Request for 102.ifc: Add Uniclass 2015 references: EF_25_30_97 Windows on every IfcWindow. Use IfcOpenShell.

First a look at what the model holds.

```python
import ifcopenshell

model = ifcopenshell.open("102.ifc")
print(model.schema)
print("classifications:", [c.Name for c in model.by_type("IfcClassification")])
for ifc_class in ("IfcDoor", "IfcRoof", "IfcStair", "IfcWall", "IfcWindow"):
    print(ifc_class, len(model.by_type(ifc_class)))
```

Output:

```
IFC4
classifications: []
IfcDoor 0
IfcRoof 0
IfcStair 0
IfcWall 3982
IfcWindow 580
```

```python
import ifcopenshell
import ifcopenshell.api.classification

model = ifcopenshell.open("102.ifc")

system = ifcopenshell.api.classification.add_classification(model, classification="Uniclass 2015")

codes = {
    "IfcWindow": ("EF_25_30_97", "Windows"),
}
for ifc_class, (code, name) in codes.items():
    products = model.by_type(ifc_class)
    ifcopenshell.api.classification.add_reference(
        model, products=products, classification=system, identification=code, name=name
    )
    print(code, len(products))

model.write("102_rev.ifc")
```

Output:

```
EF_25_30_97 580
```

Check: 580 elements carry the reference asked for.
